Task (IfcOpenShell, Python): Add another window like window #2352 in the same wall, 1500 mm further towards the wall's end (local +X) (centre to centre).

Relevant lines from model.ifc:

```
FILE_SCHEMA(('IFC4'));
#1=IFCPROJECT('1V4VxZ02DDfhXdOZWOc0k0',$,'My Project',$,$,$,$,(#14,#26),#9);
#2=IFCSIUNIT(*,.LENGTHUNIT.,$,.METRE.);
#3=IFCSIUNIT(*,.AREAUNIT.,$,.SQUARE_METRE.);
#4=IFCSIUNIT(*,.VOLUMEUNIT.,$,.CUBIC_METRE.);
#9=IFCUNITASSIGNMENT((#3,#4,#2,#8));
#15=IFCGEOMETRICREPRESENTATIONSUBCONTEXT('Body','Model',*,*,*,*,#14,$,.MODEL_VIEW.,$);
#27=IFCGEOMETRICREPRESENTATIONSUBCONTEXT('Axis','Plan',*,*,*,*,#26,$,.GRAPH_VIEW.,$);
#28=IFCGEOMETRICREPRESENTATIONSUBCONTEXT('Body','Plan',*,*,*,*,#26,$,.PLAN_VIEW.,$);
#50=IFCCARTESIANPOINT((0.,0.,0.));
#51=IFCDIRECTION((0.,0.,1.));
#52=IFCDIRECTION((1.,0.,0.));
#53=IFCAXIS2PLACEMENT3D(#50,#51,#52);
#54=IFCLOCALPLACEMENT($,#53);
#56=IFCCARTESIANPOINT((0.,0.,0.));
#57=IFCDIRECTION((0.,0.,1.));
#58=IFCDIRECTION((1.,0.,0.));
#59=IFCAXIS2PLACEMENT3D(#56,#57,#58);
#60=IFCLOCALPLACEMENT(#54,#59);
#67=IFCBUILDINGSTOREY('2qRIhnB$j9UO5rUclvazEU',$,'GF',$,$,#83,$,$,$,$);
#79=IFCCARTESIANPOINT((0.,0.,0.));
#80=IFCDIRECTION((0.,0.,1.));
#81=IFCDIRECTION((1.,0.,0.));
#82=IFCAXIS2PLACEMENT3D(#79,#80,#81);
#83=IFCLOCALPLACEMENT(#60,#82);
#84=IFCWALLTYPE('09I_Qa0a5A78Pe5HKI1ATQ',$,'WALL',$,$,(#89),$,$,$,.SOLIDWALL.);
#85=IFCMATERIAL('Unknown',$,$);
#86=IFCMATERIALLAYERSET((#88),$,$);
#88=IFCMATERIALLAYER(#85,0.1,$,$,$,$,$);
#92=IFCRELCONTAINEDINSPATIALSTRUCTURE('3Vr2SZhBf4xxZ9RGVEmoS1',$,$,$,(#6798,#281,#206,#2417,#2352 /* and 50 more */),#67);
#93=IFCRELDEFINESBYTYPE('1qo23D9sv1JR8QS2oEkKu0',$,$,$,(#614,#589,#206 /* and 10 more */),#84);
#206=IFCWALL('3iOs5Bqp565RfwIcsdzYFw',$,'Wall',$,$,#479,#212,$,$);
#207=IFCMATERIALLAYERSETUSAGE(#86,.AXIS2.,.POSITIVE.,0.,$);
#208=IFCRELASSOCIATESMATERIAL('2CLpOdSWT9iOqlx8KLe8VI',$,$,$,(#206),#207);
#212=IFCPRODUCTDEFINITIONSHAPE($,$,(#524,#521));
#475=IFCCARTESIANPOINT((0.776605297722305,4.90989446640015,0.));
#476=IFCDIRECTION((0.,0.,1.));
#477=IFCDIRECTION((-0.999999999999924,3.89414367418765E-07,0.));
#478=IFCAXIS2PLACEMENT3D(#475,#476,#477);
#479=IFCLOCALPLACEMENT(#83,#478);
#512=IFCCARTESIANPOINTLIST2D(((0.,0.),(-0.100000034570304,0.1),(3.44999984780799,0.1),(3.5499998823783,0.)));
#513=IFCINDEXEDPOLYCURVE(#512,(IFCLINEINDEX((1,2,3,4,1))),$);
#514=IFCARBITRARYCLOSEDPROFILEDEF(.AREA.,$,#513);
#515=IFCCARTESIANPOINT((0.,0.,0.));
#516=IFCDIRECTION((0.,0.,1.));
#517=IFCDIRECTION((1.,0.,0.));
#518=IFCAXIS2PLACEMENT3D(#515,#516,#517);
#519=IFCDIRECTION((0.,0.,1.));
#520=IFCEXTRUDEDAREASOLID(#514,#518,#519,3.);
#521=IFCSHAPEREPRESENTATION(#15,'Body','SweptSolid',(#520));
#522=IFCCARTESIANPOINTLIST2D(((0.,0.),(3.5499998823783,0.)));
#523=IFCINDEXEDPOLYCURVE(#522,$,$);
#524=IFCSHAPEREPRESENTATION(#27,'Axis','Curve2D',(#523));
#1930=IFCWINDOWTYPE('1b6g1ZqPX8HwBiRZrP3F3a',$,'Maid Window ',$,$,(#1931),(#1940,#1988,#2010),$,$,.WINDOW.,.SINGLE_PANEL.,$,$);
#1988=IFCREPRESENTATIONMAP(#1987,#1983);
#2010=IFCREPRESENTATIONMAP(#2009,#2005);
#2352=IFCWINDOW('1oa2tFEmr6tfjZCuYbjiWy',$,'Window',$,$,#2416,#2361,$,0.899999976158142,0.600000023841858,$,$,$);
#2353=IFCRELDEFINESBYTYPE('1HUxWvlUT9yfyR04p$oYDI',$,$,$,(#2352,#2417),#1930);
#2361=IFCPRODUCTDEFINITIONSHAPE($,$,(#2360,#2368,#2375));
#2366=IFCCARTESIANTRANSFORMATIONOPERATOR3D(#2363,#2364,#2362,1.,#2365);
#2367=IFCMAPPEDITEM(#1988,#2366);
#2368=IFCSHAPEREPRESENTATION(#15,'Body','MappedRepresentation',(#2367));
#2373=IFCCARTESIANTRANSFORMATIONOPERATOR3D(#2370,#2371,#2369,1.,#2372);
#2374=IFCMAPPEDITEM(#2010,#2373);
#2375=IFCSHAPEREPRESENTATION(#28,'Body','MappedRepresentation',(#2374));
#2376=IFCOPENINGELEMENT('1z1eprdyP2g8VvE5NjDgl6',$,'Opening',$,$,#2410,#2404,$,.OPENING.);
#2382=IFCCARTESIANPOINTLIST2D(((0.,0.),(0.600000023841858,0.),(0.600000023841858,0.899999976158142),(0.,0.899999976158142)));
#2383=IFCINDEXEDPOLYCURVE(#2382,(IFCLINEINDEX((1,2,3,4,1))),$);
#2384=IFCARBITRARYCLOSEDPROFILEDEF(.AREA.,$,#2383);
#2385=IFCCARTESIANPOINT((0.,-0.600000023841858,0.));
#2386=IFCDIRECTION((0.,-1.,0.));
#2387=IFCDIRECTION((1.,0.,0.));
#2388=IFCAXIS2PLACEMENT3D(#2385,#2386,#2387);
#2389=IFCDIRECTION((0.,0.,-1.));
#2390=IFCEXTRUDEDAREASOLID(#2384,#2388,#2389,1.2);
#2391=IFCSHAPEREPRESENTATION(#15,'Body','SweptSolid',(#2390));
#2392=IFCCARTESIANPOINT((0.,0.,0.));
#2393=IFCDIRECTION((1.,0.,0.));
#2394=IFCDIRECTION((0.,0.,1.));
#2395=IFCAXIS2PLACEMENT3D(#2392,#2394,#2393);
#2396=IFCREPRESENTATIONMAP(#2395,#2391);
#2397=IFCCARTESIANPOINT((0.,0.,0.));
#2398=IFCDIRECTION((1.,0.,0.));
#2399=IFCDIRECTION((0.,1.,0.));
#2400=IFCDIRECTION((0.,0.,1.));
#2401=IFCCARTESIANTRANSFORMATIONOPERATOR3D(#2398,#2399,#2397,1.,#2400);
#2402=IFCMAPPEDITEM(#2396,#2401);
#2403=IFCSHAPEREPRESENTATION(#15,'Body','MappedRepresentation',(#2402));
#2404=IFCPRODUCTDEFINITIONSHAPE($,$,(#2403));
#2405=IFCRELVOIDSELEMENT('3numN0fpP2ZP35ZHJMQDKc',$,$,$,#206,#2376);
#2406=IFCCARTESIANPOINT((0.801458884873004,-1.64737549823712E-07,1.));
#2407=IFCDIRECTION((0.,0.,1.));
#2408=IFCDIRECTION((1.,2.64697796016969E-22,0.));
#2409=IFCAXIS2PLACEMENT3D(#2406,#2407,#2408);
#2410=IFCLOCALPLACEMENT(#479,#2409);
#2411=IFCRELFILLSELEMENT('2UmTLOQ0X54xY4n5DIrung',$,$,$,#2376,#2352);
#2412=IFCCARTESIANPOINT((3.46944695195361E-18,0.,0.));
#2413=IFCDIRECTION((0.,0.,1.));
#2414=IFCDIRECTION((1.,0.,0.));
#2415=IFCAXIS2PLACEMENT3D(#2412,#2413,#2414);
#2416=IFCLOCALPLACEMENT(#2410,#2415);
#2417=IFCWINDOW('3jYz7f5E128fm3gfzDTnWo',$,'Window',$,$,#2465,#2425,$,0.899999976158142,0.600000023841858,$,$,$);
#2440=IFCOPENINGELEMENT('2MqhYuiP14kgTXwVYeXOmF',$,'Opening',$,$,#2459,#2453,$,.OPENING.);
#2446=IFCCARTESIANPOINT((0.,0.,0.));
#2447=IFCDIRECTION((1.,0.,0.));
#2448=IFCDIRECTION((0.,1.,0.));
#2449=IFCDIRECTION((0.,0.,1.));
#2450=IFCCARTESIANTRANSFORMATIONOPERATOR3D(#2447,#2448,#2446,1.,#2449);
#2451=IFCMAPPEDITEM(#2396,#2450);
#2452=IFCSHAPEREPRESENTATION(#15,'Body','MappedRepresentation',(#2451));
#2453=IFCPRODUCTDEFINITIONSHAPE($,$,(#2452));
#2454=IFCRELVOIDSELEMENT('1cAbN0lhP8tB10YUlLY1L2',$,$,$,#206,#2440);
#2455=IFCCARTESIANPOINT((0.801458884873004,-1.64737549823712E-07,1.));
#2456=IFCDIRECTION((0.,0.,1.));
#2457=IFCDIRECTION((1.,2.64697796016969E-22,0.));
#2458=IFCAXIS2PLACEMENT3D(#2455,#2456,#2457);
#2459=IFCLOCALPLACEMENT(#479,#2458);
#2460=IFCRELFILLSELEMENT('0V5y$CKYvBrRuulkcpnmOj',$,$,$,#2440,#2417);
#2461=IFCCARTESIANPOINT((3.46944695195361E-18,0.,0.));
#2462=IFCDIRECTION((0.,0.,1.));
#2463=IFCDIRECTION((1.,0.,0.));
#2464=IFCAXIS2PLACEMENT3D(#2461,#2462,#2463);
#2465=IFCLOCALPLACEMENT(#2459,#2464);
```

```python
import ifcopenshell
import ifcopenshell.api.feature
import ifcopenshell.api.geometry
import ifcopenshell.api.root
import ifcopenshell.geom
import ifcopenshell.util.element
import ifcopenshell.util.placement
import ifcopenshell.util.shape

model = ifcopenshell.open("model.ifc")
settings = ifcopenshell.geom.settings()


def volume(element):
    """Net volume in cubic metres, openings subtracted."""
    shape = ifcopenshell.geom.create_shape(settings, element)
    return ifcopenshell.util.shape.get_volume(shape.geometry)


window = model.by_guid("1oa2tFEmr6tfjZCuYbjiWy")
opening = window.FillsVoids[0].RelatingOpeningElement
wall = opening.VoidsElements[0].RelatingBuildingElement
before = volume(wall)
shift = ifcopenshell.util.placement.get_local_placement(wall.ObjectPlacement)[:3, 0] * 1.5

# copy_class copies the void relationship, type, container and properties, but no geometry.
new_opening = ifcopenshell.api.root.copy_class(model, product=opening)
new_opening.Representation = ifcopenshell.util.element.copy_deep(
    model, opening.Representation, exclude=["IfcGeometricRepresentationContext", "IfcRepresentationMap"]
)
new_window = ifcopenshell.api.root.copy_class(model, product=window)
new_window.Representation = ifcopenshell.util.element.copy_deep(
    model, window.Representation, exclude=["IfcGeometricRepresentationContext", "IfcRepresentationMap"]
)
ifcopenshell.api.feature.add_filling(model, opening=new_opening, element=new_window)

for old, new in ((opening, new_opening), (window, new_window)):
    matrix = ifcopenshell.util.placement.get_local_placement(old.ObjectPlacement)
    matrix[:3, 3] += shift
    ifcopenshell.api.geometry.edit_object_placement(model, product=new, matrix=matrix, is_si=False)

after = volume(wall)

print(f"wall volume {before:.3f} -> {after:.3f} m3")

model.write("model_edited.ifc")
```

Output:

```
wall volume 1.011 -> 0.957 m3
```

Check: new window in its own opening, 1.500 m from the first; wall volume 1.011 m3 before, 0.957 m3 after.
